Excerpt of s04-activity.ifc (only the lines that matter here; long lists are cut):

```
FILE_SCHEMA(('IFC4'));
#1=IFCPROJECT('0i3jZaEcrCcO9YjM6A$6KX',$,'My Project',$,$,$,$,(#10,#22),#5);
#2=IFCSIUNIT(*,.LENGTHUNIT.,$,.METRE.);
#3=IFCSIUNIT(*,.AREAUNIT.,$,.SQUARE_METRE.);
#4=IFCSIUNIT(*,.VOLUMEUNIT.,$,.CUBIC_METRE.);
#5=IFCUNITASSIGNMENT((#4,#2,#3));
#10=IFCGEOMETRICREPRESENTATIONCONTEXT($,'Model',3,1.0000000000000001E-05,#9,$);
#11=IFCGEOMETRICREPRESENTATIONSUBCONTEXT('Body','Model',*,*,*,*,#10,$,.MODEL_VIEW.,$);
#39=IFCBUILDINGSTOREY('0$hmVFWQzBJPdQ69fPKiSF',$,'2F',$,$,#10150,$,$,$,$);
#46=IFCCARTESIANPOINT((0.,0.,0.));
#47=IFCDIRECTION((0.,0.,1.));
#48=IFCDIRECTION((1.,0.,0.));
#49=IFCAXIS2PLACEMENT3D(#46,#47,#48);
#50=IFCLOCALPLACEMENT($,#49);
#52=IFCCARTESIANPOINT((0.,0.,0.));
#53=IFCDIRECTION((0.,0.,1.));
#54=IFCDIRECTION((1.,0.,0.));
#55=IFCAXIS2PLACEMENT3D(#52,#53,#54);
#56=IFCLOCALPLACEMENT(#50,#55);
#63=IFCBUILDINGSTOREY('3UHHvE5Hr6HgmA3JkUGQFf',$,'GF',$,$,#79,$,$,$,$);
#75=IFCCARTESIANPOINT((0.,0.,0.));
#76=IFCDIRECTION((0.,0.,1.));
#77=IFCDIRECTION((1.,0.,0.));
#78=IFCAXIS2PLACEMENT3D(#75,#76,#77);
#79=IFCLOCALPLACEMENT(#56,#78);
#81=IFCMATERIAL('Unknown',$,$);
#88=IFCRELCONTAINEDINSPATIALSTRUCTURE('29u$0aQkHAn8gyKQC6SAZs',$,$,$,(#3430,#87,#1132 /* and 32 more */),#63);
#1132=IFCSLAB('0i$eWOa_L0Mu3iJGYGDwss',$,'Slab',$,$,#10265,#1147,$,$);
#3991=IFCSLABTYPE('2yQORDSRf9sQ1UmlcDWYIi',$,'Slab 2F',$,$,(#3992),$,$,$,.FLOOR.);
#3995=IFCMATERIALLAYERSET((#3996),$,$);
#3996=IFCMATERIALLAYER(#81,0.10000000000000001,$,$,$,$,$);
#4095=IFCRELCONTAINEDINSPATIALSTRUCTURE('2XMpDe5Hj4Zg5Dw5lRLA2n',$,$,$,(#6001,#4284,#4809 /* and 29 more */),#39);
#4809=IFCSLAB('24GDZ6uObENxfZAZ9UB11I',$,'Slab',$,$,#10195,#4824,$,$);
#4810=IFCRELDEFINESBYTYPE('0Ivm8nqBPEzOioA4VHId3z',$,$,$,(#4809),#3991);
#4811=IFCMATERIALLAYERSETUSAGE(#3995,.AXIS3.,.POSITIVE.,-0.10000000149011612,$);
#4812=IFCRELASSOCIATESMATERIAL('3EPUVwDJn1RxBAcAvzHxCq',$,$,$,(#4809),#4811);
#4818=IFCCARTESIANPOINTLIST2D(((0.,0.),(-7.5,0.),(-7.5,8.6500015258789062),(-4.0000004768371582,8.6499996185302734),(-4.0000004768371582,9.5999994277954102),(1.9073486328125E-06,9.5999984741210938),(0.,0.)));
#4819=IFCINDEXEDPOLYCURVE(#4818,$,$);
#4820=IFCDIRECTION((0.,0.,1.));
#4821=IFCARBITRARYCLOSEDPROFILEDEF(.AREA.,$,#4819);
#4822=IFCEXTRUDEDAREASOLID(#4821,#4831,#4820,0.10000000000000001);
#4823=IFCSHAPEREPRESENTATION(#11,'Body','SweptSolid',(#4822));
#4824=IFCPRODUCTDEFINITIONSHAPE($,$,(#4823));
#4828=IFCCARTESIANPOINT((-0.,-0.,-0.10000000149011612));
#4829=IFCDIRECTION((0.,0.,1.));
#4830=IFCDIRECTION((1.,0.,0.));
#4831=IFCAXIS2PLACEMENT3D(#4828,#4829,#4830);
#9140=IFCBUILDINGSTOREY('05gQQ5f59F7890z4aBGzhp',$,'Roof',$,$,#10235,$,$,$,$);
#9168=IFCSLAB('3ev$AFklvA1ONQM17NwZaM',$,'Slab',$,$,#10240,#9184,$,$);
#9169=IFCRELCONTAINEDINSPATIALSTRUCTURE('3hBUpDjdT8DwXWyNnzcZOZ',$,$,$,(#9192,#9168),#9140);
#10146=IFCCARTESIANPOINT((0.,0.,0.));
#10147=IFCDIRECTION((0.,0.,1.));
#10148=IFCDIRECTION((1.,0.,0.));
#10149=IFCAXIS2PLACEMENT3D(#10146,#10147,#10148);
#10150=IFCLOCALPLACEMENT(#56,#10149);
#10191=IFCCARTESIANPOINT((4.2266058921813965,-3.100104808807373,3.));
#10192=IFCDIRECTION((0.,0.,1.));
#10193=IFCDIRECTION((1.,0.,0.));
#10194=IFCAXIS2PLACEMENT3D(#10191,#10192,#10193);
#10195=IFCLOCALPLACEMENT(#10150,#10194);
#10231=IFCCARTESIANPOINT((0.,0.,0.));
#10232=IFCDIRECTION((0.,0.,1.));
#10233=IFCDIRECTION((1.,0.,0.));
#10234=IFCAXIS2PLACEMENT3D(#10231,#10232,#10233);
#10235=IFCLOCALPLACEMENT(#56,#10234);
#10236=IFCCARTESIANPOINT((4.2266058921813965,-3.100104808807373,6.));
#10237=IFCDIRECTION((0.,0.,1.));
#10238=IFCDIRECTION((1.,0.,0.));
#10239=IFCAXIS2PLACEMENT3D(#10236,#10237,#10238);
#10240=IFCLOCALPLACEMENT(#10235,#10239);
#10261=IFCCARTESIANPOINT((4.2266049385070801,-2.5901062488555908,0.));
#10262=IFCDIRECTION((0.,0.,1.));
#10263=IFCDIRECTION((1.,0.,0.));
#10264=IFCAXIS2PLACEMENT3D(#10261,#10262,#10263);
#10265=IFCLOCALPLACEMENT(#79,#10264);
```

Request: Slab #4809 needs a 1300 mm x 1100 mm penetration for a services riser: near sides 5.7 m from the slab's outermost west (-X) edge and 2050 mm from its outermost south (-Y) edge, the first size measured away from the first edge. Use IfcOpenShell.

```python
import numpy as np
import ifcopenshell
import ifcopenshell.api.feature
import ifcopenshell.api.geometry
import ifcopenshell.api.root
import ifcopenshell.geom
import ifcopenshell.util.placement
import ifcopenshell.util.representation
import ifcopenshell.util.shape
import ifcopenshell.util.unit

model = ifcopenshell.open("s04-activity.ifc")
unit_scale = ifcopenshell.util.unit.calculate_unit_scale(model)
settings = ifcopenshell.geom.settings()


def volume(element):
    """Net volume in cubic metres, openings subtracted."""
    shape = ifcopenshell.geom.create_shape(settings, element)
    return ifcopenshell.util.shape.get_volume(shape.geometry)


slab = model.by_guid("24GDZ6uObENxfZAZ9UB11I")
before = volume(slab)

# Extent in the slab's own axes, in metres. The edges named are its -X and -Y sides.
slab_shape = ifcopenshell.geom.create_shape(settings, slab)
vertices = ifcopenshell.util.shape.get_vertices(slab_shape.geometry)
x_min, y_min, bottom = vertices.min(axis=0)
top = vertices[:, 2].max()

opening = ifcopenshell.api.root.create_entity(model, ifc_class="IfcOpeningElement", name="Services riser opening", predefined_type="OPENING")
context = ifcopenshell.util.representation.get_context(model, "Model", "Body", "MODEL_VIEW")
width, depth = 1.3, 1.1
outline = [(0.0, 0.0), (width, 0.0), (width, depth), (0.0, depth), (0.0, 0.0)]
# Overshoot both faces by 50 mm so the cut is clean.
shape = ifcopenshell.api.geometry.add_slab_representation(
    model, context=context, depth=top - bottom + 0.1, polyline=outline
)
ifcopenshell.api.geometry.assign_representation(model, product=opening, representation=shape)

matrix = ifcopenshell.util.placement.get_local_placement(slab.ObjectPlacement)
matrix[:, 3] = matrix @ np.append(np.array([x_min + 5.7, y_min + 2.05, bottom - 0.05]) / unit_scale, 1.0)
ifcopenshell.api.geometry.edit_object_placement(model, product=opening, matrix=matrix, is_si=False)
ifcopenshell.api.feature.add_feature(model, feature=opening, element=slab)

after = volume(slab)

print(f"slab volume {before:.3f} -> {after:.3f} m3")

model.write("s04-activity_v2.ifc")
```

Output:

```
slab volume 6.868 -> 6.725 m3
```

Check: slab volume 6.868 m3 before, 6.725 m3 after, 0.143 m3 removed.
